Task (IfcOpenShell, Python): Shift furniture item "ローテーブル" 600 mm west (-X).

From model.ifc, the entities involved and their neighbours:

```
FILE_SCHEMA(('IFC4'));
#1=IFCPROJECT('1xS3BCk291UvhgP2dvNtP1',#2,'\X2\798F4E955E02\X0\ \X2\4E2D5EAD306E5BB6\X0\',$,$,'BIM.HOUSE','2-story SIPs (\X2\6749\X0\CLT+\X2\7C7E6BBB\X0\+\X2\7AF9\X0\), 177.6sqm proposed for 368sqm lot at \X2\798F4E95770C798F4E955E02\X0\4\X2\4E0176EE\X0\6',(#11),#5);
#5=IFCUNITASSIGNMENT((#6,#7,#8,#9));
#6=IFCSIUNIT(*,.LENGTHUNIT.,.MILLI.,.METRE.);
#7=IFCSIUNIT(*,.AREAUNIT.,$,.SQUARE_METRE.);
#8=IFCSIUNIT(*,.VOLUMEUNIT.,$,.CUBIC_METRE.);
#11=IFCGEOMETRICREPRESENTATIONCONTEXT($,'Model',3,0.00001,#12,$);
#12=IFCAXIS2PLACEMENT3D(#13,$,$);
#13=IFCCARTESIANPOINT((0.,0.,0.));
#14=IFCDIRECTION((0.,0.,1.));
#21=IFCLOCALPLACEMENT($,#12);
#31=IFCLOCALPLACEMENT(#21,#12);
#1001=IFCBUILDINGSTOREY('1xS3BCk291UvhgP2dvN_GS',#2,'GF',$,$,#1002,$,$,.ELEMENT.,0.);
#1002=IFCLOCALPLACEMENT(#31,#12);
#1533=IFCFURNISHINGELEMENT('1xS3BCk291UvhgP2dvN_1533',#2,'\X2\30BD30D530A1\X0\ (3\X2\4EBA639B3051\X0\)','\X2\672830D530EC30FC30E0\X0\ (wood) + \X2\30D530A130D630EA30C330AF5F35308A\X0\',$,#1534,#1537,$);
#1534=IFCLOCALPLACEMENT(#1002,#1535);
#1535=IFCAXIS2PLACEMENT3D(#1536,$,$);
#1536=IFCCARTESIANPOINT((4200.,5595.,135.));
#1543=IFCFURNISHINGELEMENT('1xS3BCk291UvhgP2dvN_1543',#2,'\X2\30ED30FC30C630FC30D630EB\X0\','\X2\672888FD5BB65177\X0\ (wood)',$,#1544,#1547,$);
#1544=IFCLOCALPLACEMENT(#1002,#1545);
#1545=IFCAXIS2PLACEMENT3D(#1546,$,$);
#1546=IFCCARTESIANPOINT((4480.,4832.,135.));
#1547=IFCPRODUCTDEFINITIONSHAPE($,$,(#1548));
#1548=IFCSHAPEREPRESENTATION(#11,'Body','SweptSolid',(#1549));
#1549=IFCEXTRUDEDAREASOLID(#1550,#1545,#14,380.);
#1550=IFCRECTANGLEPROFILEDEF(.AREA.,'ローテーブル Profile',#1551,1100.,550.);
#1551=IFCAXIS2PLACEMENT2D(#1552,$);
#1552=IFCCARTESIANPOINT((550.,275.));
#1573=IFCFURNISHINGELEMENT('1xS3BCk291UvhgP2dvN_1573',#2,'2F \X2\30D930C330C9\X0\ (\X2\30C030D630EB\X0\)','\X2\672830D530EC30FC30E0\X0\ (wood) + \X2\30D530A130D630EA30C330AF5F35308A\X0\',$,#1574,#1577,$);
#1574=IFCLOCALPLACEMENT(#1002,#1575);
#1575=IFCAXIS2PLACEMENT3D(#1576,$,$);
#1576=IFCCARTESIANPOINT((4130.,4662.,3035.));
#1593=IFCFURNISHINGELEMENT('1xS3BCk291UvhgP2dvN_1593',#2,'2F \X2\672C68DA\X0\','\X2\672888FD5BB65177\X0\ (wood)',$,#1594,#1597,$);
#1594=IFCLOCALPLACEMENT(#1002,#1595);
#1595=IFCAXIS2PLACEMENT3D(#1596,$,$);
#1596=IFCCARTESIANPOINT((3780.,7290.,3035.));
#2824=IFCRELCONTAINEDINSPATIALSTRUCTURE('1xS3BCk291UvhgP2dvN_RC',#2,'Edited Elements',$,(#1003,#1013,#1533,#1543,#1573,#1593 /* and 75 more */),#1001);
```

```python
import ifcopenshell
import ifcopenshell.api.geometry
import ifcopenshell.util.placement
import ifcopenshell.util.unit

model = ifcopenshell.open("model.ifc")
unit_scale = ifcopenshell.util.unit.calculate_unit_scale(model)

item = model.by_guid("1xS3BCk291UvhgP2dvN_1543")
matrix = ifcopenshell.util.placement.get_local_placement(item.ObjectPlacement)
matrix[0, 3] -= 0.6 / unit_scale
ifcopenshell.api.geometry.edit_object_placement(model, product=item, matrix=matrix, is_si=False)

print(ifcopenshell.util.placement.get_local_placement(item.ObjectPlacement).round(3) + 0.0)

model.write("model_v2.ifc")
```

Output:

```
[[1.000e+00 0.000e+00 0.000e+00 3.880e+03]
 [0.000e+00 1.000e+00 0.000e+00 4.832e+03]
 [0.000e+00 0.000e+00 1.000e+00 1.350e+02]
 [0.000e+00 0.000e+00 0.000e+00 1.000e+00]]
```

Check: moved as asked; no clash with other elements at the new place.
